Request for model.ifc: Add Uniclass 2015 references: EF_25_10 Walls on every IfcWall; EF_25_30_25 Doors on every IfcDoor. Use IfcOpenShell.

First a look at what the model holds.

```python
import ifcopenshell

model = ifcopenshell.open("model.ifc")
print(model.schema)
print("classifications:", [c.Name for c in model.by_type("IfcClassification")])
for ifc_class in ("IfcDoor", "IfcRoof", "IfcStair", "IfcWall", "IfcWindow"):
    print(ifc_class, len(model.by_type(ifc_class)))
```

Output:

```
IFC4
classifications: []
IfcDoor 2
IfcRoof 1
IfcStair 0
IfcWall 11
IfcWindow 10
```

```python
import ifcopenshell
import ifcopenshell.api.classification

model = ifcopenshell.open("model.ifc")

system = ifcopenshell.api.classification.add_classification(model, classification="Uniclass 2015")

codes = {
    "IfcWall": ("EF_25_10", "Walls"),
    "IfcDoor": ("EF_25_30_25", "Doors"),
}
for ifc_class, (code, name) in codes.items():
    products = model.by_type(ifc_class)
    ifcopenshell.api.classification.add_reference(
        model, products=products, classification=system, identification=code, name=name
    )
    print(code, len(products))

model.write("model_v2.ifc")
```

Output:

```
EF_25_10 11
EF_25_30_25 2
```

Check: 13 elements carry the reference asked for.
